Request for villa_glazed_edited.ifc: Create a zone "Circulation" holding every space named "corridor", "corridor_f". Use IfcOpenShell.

First a look at what the model holds.

```python
import ifcopenshell

model = ifcopenshell.open("villa_glazed_edited.ifc")
print(model.schema)
seen = {}
for space in model.by_type("IfcSpace"):
    seen[space.LongName] = seen.get(space.LongName, 0) + 1
for name, count in sorted(seen.items(), key=str):
    print(count, "x", name)
print("zones:", [z.Name for z in model.by_type("IfcZone")][:20])
```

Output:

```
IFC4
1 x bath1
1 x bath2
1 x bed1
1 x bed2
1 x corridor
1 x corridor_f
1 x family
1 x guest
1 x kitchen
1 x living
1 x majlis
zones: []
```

```python
import ifcopenshell
import ifcopenshell.api.group
import ifcopenshell.api.root

model = ifcopenshell.open("villa_glazed_edited.ifc")

names = {"corridor", "corridor_f"}
spaces = [s for s in model.by_type("IfcSpace") if s.LongName in names]

zone = ifcopenshell.api.root.create_entity(model, ifc_class="IfcZone", name="Circulation")
ifcopenshell.api.group.assign_group(model, products=spaces, group=zone)
print(len(spaces), "spaces in", zone.Name)

model.write("villa_glazed_edited_edited.ifc")
```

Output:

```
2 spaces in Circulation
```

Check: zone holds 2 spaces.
